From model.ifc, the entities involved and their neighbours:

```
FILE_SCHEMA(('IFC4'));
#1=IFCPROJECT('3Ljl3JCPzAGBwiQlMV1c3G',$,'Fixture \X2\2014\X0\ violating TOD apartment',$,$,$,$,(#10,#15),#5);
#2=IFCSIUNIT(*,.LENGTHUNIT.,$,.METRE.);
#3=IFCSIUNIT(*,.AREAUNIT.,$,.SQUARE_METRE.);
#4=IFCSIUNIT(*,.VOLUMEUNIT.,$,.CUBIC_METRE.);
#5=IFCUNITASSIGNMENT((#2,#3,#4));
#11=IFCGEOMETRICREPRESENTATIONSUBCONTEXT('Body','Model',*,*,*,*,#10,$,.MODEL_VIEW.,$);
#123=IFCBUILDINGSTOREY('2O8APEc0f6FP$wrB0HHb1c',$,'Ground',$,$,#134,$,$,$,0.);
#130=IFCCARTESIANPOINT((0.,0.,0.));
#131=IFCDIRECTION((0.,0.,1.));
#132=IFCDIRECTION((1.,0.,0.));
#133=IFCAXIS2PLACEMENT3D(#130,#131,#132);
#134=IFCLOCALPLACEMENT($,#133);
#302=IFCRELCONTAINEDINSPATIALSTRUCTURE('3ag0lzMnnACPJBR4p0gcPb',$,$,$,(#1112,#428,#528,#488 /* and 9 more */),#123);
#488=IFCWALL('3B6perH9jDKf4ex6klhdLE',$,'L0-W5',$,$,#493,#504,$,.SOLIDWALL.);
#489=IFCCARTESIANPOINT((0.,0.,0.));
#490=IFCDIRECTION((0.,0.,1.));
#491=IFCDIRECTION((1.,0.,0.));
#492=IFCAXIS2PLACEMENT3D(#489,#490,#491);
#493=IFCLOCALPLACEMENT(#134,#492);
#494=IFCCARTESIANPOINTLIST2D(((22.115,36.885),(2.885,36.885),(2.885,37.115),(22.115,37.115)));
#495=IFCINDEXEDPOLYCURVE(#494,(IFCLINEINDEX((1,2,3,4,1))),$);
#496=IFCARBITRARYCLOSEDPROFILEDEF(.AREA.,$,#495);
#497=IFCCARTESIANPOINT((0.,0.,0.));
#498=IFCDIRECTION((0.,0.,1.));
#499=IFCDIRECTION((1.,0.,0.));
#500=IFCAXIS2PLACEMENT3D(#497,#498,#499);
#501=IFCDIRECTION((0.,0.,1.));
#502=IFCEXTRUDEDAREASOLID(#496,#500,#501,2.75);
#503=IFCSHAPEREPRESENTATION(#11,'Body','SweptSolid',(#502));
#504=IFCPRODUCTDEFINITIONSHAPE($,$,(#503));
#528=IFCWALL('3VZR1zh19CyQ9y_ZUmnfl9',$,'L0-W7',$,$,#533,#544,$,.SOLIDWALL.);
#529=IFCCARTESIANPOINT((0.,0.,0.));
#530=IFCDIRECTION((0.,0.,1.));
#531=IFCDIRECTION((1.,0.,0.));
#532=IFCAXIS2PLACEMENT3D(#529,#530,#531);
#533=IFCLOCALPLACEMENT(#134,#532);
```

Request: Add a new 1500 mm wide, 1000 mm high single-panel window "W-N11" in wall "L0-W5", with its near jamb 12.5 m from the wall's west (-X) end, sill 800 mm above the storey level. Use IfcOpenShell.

```python
import numpy as np
import ifcopenshell
import ifcopenshell.api.feature
import ifcopenshell.api.geometry
import ifcopenshell.api.root
import ifcopenshell.api.spatial
import ifcopenshell.geom
import ifcopenshell.util.element
import ifcopenshell.util.placement
import ifcopenshell.util.representation
import ifcopenshell.util.shape
import ifcopenshell.util.unit

model = ifcopenshell.open("model.ifc")
unit_scale = ifcopenshell.util.unit.calculate_unit_scale(model)
settings = ifcopenshell.geom.settings()


def volume(element):
    """Net volume in cubic metres, openings subtracted."""
    shape = ifcopenshell.geom.create_shape(settings, element)
    return ifcopenshell.util.shape.get_volume(shape.geometry)


wall = model.by_guid("3B6perH9jDKf4ex6klhdLE")
storey = ifcopenshell.util.element.get_container(wall, ifc_class="IfcBuildingStorey")
context = ifcopenshell.util.representation.get_context(model, "Model", "Body", "MODEL_VIEW")
before = volume(wall)

width, height, from_end, sill = 1.5, 1, 12.5, 0.8  # metres

# The wall runs along its own X axis, and the end named is its -X end.
wall_shape = ifcopenshell.geom.create_shape(settings, wall)
x, y, z = ifcopenshell.util.shape.get_vertices(wall_shape.geometry).T
start = x.min() + from_end
face, thickness = float(y.min()), float(y.max() - y.min())
wall_matrix = ifcopenshell.util.placement.get_local_placement(wall.ObjectPlacement)
level = ifcopenshell.util.placement.get_local_placement(storey.ObjectPlacement)[2, 3]


def in_wall(x, y):
    """Placement at x, y metres in the wall's axes, at sill height."""
    matrix = wall_matrix.copy()
    matrix[:, 3] = wall_matrix @ np.array([x / unit_scale, y / unit_scale, 0.0, 1.0])
    matrix[2, 3] = level + sill / unit_scale
    return matrix


# Opening: a box that overshoots both wall faces by 50 mm.
opening = ifcopenshell.api.root.create_entity(model, ifc_class="IfcOpeningElement", predefined_type="OPENING")
box = ifcopenshell.api.geometry.add_wall_representation(
    model, context=context, length=width, height=height, thickness=thickness + 0.1
)
ifcopenshell.api.geometry.assign_representation(model, product=opening, representation=box)
ifcopenshell.api.geometry.edit_object_placement(model, product=opening, matrix=in_wall(start, face - 0.05), is_si=False)
ifcopenshell.api.feature.add_feature(model, feature=opening, element=wall)

window = ifcopenshell.api.root.create_entity(model, ifc_class="IfcWindow", name="W-N11", predefined_type="WINDOW")
window.OverallWidth, window.OverallHeight = width / unit_scale, height / unit_scale
window.PartitioningType = "SINGLE_PANEL"
body = ifcopenshell.api.geometry.add_window_representation(
    model,
    context=context,
    overall_width=window.OverallWidth,
    overall_height=window.OverallHeight,
    partition_type="SINGLE_PANEL",
)
ifcopenshell.api.geometry.assign_representation(model, product=window, representation=body)
ifcopenshell.api.spatial.assign_container(model, products=[window], relating_structure=storey)
ifcopenshell.api.feature.add_filling(model, opening=opening, element=window)

# Centre the window in the wall's thickness.
ifcopenshell.api.geometry.edit_object_placement(model, product=window, matrix=in_wall(start, face), is_si=False)
window_shape = ifcopenshell.geom.create_shape(settings, window)
depth = ifcopenshell.util.shape.get_vertices(window_shape.geometry)[:, 1]
offset = face + thickness / 2 - (depth.min() + depth.max()) / 2
ifcopenshell.api.geometry.edit_object_placement(model, product=window, matrix=in_wall(start, offset), is_si=False)

after = volume(wall)

print(f"wall volume {before:.3f} -> {after:.3f} m3")

model.write("model_edited.ifc")
```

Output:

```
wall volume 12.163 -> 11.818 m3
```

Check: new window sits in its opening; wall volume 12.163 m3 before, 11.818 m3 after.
